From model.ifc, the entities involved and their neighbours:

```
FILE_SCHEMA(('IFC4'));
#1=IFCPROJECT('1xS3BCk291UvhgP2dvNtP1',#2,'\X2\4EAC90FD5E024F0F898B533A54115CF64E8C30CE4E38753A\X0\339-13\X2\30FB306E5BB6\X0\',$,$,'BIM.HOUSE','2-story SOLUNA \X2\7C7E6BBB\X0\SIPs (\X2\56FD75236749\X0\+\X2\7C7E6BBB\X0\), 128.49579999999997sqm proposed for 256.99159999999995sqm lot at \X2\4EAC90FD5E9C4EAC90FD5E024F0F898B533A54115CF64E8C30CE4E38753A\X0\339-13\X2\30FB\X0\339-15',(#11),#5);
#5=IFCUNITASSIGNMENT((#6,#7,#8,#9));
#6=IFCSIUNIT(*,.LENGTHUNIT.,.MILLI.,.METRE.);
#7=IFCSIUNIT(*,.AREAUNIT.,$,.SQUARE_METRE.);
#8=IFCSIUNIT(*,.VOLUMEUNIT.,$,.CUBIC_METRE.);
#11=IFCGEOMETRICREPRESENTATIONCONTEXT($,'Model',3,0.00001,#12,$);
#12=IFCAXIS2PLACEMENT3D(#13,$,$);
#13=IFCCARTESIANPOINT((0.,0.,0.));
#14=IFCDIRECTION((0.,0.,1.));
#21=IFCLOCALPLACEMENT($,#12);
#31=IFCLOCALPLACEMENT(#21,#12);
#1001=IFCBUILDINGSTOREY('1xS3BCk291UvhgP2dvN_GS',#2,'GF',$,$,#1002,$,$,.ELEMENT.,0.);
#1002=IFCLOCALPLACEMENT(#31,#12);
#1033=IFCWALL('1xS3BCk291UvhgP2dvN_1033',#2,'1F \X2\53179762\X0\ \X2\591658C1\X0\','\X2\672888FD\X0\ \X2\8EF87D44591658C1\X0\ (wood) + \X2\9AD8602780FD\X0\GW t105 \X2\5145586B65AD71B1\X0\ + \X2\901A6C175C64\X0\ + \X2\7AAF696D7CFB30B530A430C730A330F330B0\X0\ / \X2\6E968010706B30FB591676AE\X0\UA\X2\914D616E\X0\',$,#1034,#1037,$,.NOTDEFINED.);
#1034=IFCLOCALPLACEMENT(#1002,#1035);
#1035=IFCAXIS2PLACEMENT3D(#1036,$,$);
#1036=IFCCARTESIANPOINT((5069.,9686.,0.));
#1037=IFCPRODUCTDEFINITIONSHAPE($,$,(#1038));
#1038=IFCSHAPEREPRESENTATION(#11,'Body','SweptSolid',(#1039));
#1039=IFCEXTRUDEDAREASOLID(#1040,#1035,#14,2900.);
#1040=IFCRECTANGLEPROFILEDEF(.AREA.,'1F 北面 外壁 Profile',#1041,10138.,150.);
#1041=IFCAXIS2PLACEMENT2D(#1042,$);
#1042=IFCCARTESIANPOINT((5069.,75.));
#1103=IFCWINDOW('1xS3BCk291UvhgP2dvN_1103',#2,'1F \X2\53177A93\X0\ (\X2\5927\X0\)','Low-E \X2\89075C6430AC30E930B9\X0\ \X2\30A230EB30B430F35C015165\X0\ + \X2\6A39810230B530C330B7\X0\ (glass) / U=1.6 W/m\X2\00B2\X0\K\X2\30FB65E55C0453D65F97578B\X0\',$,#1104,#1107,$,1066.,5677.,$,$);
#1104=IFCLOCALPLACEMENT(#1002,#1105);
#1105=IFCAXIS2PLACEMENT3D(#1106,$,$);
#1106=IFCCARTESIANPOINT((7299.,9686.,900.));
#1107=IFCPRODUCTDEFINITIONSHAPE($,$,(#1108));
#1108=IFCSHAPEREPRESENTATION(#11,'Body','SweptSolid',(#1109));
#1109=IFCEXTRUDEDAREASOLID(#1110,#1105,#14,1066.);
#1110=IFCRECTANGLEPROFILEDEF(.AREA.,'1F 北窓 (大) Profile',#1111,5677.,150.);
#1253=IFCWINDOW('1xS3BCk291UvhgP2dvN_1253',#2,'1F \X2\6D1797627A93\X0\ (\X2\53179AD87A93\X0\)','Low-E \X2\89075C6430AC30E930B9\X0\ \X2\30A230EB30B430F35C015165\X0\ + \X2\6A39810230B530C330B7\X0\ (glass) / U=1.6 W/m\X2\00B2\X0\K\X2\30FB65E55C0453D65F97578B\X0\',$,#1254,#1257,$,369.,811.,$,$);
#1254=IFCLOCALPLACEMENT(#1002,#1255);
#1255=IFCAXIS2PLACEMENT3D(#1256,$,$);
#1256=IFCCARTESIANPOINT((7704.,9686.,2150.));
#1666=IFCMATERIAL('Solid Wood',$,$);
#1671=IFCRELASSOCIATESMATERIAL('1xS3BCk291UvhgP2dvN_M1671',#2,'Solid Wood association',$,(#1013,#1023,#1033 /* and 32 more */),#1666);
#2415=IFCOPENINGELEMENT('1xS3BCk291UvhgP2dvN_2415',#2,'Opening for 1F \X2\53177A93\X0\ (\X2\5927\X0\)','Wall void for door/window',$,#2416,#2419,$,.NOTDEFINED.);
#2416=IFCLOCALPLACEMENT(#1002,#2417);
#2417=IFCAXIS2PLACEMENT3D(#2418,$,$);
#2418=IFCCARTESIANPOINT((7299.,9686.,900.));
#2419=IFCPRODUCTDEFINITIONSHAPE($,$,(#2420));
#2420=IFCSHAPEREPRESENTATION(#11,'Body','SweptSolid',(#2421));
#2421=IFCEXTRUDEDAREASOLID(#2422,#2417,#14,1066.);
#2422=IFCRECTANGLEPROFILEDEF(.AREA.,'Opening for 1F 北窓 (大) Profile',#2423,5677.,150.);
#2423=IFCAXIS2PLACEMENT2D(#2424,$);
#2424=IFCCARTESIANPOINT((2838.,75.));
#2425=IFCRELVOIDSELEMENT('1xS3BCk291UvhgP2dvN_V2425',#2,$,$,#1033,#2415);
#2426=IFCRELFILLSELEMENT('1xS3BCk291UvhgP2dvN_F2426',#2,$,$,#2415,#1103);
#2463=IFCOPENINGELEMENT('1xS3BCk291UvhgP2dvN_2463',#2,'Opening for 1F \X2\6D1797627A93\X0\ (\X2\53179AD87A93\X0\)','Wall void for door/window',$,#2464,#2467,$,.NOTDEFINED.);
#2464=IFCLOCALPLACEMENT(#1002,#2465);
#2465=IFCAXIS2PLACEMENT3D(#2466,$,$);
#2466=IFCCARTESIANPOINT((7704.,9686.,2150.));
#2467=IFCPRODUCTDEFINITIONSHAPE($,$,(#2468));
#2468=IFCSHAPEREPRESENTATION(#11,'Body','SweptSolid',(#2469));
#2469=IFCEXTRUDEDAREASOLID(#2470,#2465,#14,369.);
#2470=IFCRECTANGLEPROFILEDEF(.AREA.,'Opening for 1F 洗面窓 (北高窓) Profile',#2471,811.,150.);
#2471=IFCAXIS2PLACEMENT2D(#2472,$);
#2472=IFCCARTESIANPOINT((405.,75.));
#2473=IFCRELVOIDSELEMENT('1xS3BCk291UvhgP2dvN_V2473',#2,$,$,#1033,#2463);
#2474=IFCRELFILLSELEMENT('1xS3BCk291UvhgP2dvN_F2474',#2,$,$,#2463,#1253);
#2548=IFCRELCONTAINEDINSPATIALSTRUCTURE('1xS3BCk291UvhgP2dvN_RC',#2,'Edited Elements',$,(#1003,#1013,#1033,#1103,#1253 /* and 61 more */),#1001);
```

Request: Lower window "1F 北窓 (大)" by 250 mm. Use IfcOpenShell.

```python
import numpy as np
import ifcopenshell
import ifcopenshell.api.geometry
import ifcopenshell.util.placement
import ifcopenshell.util.unit

model = ifcopenshell.open("model.ifc")
unit_scale = ifcopenshell.util.unit.calculate_unit_scale(model)

window = model.by_guid("1xS3BCk291UvhgP2dvN_1103")
opening = window.FillsVoids[0].RelatingOpeningElement
dz = -0.25 / unit_scale

shift = np.array([0.0, 0.0, dz])
# The window is not placed relative to its opening, so move both.
for product in (opening, window):
    matrix = ifcopenshell.util.placement.get_local_placement(product.ObjectPlacement)
    matrix[:3, 3] += shift
    ifcopenshell.api.geometry.edit_object_placement(model, product=product, matrix=matrix, is_si=False)

print(f"moved by {dz * unit_scale:+.3f} m")

model.write("model_v2.ifc")
```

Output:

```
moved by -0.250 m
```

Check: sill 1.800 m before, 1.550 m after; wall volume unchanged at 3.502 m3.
